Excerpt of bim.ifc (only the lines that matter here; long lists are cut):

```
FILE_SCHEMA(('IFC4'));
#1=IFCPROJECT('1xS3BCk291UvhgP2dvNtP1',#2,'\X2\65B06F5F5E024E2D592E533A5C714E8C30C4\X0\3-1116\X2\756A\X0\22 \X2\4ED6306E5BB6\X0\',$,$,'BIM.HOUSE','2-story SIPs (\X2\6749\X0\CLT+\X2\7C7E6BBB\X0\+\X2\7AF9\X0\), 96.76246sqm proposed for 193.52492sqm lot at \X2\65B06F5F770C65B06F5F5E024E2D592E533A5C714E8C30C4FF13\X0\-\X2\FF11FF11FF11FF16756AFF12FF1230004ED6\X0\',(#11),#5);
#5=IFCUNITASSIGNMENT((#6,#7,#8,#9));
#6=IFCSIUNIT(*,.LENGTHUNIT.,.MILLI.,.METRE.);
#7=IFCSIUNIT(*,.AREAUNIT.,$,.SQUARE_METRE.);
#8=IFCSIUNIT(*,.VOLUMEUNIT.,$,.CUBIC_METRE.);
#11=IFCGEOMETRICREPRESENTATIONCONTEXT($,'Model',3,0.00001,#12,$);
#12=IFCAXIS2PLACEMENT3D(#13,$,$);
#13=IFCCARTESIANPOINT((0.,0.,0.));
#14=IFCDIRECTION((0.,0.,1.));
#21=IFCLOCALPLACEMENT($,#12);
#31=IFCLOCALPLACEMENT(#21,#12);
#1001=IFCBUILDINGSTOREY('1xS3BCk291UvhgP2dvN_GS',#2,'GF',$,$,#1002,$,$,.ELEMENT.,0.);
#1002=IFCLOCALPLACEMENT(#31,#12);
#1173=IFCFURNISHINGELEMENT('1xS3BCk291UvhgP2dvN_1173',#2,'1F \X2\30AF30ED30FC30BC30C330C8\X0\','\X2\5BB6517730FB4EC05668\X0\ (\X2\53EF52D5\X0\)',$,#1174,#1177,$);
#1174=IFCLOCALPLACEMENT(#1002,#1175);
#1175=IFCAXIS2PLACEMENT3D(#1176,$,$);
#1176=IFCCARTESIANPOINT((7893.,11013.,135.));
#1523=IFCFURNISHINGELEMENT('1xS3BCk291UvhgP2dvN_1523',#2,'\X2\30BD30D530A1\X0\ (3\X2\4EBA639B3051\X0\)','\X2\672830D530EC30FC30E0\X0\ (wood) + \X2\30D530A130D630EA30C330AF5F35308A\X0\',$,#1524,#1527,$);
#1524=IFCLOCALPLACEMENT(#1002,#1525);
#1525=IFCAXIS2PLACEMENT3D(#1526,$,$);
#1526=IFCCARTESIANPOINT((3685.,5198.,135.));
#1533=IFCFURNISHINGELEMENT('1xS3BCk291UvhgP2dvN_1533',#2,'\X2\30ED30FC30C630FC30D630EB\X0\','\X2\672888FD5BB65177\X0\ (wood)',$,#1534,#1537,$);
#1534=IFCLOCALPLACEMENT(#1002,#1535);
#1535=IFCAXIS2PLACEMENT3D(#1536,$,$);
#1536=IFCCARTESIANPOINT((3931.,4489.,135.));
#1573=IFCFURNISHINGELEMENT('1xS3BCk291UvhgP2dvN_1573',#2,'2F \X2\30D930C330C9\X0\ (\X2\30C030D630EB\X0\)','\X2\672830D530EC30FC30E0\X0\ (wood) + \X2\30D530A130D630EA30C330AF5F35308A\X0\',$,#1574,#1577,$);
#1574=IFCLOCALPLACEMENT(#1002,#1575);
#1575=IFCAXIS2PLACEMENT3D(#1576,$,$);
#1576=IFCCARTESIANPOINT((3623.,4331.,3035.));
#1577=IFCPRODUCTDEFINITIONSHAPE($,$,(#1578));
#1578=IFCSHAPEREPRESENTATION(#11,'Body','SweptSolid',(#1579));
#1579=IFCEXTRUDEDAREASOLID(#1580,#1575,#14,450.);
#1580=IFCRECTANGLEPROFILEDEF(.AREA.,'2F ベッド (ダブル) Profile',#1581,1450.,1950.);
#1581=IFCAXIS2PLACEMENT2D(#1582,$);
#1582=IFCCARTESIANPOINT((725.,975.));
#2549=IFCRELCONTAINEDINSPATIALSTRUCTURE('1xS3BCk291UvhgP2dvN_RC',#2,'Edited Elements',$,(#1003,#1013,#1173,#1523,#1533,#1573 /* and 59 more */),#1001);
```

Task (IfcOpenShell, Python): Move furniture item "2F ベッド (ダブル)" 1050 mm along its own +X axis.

```python
import ifcopenshell
import ifcopenshell.api.geometry
import ifcopenshell.util.placement

model = ifcopenshell.open("bim.ifc")

item = model.by_guid("1xS3BCk291UvhgP2dvN_1573")
matrix = ifcopenshell.util.placement.get_local_placement(item.ObjectPlacement)
matrix[:3, 3] += matrix[:3, 0] * 1050.0
ifcopenshell.api.geometry.edit_object_placement(model, product=item, matrix=matrix, is_si=False)

print(ifcopenshell.util.placement.get_local_placement(item.ObjectPlacement).round(3) + 0.0)

model.write("bim-out.ifc")
```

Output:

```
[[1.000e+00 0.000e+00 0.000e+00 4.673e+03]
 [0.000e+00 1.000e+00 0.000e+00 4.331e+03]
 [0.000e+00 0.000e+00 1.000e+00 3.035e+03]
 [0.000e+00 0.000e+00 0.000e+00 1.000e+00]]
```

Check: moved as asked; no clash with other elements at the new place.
